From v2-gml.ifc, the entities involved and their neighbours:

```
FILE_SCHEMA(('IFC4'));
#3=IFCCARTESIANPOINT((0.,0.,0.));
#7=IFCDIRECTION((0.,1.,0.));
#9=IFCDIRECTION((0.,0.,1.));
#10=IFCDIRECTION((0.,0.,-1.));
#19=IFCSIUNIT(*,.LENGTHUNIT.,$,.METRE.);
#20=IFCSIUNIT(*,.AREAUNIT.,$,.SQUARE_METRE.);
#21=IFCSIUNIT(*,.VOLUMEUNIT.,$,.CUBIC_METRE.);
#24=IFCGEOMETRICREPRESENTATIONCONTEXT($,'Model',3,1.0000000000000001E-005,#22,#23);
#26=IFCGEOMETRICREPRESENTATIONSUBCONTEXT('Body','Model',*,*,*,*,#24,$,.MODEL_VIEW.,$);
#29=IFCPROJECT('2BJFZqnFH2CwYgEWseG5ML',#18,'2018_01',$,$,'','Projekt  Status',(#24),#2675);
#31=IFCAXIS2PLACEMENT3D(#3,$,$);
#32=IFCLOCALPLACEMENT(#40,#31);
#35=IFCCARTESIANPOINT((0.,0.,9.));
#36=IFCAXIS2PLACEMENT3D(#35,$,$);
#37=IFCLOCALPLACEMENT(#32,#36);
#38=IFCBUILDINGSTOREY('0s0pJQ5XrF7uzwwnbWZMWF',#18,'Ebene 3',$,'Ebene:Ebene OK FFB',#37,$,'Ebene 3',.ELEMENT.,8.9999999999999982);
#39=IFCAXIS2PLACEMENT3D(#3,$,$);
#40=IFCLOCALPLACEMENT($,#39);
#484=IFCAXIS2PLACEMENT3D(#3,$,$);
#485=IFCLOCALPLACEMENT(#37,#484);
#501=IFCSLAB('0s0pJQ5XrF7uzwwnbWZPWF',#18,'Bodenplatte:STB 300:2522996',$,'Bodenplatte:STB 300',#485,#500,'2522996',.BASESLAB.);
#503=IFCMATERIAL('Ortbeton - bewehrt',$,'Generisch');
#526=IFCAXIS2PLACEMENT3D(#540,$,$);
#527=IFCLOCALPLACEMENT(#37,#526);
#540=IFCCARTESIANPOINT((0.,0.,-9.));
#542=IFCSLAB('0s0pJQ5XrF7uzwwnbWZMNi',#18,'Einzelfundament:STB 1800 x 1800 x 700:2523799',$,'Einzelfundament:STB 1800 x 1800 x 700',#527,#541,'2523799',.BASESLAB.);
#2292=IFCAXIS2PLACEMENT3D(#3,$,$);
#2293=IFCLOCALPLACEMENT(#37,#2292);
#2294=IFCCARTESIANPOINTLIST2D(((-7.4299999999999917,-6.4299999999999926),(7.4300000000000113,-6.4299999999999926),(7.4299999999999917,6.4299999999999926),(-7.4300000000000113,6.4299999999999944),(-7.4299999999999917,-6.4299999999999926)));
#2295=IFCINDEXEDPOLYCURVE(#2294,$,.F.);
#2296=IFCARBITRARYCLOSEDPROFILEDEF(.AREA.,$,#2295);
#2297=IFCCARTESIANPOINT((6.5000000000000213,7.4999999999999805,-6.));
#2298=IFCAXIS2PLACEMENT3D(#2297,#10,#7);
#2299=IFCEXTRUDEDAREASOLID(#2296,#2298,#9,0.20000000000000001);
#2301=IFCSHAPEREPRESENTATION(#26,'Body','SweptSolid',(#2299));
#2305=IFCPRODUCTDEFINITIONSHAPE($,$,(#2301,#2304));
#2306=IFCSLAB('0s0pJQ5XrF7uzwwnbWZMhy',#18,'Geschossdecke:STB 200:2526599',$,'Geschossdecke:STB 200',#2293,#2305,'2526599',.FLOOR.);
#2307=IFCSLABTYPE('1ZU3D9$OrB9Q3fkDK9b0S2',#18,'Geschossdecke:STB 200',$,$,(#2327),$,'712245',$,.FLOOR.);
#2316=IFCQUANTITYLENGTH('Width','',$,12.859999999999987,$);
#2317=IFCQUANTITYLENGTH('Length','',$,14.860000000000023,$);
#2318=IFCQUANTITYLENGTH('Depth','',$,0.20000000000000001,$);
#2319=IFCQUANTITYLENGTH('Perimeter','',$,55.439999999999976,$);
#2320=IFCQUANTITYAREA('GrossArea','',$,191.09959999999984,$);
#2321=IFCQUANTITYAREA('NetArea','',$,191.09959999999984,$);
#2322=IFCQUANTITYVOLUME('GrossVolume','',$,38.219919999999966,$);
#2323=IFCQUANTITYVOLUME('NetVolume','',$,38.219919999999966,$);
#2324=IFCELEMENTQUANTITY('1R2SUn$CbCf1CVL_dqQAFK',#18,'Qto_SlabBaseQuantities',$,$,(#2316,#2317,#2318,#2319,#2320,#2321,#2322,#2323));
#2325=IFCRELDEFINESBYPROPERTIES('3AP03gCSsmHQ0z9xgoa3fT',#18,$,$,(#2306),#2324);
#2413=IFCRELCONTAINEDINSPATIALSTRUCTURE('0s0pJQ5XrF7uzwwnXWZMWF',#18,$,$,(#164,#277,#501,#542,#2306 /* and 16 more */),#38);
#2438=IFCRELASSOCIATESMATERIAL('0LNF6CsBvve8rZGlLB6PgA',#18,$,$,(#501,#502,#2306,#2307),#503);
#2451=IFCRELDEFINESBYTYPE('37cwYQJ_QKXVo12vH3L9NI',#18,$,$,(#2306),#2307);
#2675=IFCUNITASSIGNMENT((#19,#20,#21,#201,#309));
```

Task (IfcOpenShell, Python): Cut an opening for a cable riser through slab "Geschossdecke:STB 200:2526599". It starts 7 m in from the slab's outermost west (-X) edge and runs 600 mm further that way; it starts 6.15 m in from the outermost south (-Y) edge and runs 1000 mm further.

```python
import numpy as np
import ifcopenshell
import ifcopenshell.api.feature
import ifcopenshell.api.geometry
import ifcopenshell.api.pset
import ifcopenshell.api.root
import ifcopenshell.geom
import ifcopenshell.util.element
import ifcopenshell.util.placement
import ifcopenshell.util.representation
import ifcopenshell.util.shape
import ifcopenshell.util.unit

model = ifcopenshell.open("v2-gml.ifc")
unit_scale = ifcopenshell.util.unit.calculate_unit_scale(model)
area_scale = ifcopenshell.util.unit.calculate_unit_scale(model, "AREAUNIT")
volume_scale = ifcopenshell.util.unit.calculate_unit_scale(model, "VOLUMEUNIT")
settings = ifcopenshell.geom.settings()


def volume(element):
    """Net volume in cubic metres, openings subtracted."""
    shape = ifcopenshell.geom.create_shape(settings, element)
    return ifcopenshell.util.shape.get_volume(shape.geometry)


slab = model.by_guid("0s0pJQ5XrF7uzwwnbWZMhy")
before = volume(slab)

# Extent in the slab's own axes, in metres. The edges named are its -X and -Y sides.
slab_shape = ifcopenshell.geom.create_shape(settings, slab)
vertices = ifcopenshell.util.shape.get_vertices(slab_shape.geometry)
x_min, y_min, bottom = vertices.min(axis=0)
top = vertices[:, 2].max()

opening = ifcopenshell.api.root.create_entity(model, ifc_class="IfcOpeningElement", name="Cable riser opening", predefined_type="OPENING")
context = ifcopenshell.util.representation.get_context(model, "Model", "Body", "MODEL_VIEW")
width, depth = 0.6, 1
outline = [(0.0, 0.0), (width, 0.0), (width, depth), (0.0, depth), (0.0, 0.0)]
# Overshoot both faces by 50 mm so the cut is clean.
shape = ifcopenshell.api.geometry.add_slab_representation(
    model, context=context, depth=top - bottom + 0.1, polyline=outline
)
ifcopenshell.api.geometry.assign_representation(model, product=opening, representation=shape)

matrix = ifcopenshell.util.placement.get_local_placement(slab.ObjectPlacement)
matrix[:, 3] = matrix @ np.append(np.array([x_min + 7, y_min + 6.15, bottom - 0.05]) / unit_scale, 1.0)
ifcopenshell.api.geometry.edit_object_placement(model, product=opening, matrix=matrix, is_si=False)
ifcopenshell.api.feature.add_feature(model, feature=opening, element=slab)

after = volume(slab)

# Update the slab's stored quantities.
qto = model.by_id(ifcopenshell.util.element.get_pset(slab, "Qto_SlabBaseQuantities", should_inherit=False)["id"])
ifcopenshell.api.pset.edit_qto(model, qto=qto, properties={
    "NetArea": after / (top - bottom) / area_scale,
    "NetVolume": after / volume_scale,
})

print(f"slab volume {before:.3f} -> {after:.3f} m3")

model.write("v2-gml_v2.ifc")
```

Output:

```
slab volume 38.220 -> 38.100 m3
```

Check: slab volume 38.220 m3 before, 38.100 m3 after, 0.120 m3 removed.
